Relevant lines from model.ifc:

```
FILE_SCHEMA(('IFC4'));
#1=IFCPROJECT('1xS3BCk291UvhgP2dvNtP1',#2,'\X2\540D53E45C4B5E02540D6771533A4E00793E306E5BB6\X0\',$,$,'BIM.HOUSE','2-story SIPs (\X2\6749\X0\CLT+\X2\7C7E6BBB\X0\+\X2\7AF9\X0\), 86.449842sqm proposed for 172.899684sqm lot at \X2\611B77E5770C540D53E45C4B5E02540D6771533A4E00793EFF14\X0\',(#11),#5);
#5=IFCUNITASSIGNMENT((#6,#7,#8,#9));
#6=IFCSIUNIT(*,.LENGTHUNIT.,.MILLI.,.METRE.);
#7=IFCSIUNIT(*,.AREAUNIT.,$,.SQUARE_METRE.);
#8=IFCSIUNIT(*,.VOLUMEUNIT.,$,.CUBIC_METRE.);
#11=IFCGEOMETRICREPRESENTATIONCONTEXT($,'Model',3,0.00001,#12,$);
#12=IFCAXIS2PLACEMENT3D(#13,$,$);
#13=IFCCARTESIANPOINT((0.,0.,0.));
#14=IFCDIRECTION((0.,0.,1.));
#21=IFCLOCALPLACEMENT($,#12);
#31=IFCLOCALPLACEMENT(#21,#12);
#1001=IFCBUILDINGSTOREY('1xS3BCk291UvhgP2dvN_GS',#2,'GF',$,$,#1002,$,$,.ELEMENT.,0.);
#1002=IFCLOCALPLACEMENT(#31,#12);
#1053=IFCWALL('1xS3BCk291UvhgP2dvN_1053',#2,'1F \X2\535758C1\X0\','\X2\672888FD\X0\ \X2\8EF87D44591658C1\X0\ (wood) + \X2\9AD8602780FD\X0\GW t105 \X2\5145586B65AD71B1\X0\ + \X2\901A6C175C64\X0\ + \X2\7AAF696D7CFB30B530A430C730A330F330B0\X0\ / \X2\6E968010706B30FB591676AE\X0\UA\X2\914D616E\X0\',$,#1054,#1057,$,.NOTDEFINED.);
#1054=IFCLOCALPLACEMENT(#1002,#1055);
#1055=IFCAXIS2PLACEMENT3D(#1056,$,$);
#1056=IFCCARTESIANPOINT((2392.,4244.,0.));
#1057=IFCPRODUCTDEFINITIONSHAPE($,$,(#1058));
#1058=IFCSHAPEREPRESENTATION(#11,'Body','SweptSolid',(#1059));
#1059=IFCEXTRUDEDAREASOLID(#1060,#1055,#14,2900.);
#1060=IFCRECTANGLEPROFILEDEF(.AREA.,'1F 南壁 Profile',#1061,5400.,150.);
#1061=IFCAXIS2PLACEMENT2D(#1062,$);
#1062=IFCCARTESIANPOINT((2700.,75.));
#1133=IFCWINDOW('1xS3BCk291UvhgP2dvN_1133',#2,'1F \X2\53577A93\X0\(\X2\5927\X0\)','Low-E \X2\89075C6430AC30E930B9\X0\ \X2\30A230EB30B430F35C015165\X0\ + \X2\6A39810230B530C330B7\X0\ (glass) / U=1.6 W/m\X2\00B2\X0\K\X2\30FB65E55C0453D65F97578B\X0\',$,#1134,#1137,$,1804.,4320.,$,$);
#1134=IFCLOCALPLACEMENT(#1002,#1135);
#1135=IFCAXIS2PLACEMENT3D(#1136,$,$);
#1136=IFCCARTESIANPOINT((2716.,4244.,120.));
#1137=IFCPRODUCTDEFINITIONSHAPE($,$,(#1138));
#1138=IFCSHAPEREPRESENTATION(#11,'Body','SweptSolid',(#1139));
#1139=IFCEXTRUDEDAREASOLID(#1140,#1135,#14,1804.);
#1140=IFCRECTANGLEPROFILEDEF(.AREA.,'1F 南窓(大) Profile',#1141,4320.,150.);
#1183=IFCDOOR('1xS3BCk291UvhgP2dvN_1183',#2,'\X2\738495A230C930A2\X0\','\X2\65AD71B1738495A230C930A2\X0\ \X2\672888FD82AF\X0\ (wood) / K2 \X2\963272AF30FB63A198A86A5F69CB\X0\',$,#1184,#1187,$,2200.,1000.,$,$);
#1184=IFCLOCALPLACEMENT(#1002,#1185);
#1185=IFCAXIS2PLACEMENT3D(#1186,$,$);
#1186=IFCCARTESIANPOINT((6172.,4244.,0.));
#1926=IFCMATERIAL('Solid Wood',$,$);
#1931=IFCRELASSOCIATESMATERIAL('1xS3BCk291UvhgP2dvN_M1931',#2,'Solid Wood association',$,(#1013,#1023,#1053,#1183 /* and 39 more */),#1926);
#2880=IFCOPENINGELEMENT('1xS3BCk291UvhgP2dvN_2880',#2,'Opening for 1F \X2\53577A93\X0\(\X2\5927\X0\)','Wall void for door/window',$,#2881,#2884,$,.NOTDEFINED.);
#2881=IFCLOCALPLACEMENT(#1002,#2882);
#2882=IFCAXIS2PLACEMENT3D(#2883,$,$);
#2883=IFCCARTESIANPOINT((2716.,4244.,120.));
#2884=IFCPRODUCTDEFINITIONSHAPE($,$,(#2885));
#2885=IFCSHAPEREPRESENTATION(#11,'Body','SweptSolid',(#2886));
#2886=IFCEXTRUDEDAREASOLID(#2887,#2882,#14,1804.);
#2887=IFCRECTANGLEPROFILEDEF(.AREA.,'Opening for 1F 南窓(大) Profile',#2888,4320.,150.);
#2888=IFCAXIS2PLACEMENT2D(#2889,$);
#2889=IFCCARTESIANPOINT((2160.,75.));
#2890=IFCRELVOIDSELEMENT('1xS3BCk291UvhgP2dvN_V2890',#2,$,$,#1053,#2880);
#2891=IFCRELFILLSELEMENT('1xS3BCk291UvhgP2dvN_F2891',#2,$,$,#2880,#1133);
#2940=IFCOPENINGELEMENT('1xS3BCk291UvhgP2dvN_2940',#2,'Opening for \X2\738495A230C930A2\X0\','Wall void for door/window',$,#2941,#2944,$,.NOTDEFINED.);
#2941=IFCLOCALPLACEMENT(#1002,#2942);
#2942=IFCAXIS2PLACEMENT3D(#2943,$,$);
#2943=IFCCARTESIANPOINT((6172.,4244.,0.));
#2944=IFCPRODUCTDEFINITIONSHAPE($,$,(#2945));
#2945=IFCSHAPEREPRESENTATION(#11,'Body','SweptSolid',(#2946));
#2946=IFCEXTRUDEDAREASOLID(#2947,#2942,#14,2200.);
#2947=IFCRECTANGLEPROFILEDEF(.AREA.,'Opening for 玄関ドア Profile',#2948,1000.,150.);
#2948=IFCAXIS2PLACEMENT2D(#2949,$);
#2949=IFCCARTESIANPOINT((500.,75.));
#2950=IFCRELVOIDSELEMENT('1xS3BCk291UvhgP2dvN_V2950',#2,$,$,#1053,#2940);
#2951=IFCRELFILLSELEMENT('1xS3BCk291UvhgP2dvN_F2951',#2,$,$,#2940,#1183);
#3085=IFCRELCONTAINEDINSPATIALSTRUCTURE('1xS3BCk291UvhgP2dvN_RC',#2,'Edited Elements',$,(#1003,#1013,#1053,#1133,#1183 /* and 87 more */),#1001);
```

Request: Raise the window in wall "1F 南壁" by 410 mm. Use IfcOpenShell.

```python
import numpy as np
import ifcopenshell
import ifcopenshell.api.geometry
import ifcopenshell.util.placement
import ifcopenshell.util.unit

model = ifcopenshell.open("model.ifc")
unit_scale = ifcopenshell.util.unit.calculate_unit_scale(model)

window = model.by_guid("1xS3BCk291UvhgP2dvN_1133")
opening = window.FillsVoids[0].RelatingOpeningElement
dz = 0.41 / unit_scale

shift = np.array([0.0, 0.0, dz])
# The window is not placed relative to its opening, so move both.
for product in (opening, window):
    matrix = ifcopenshell.util.placement.get_local_placement(product.ObjectPlacement)
    matrix[:3, 3] += shift
    ifcopenshell.api.geometry.edit_object_placement(model, product=product, matrix=matrix, is_si=False)

print(f"moved by {dz * unit_scale:+.3f} m")

model.write("model_edited.ifc")
```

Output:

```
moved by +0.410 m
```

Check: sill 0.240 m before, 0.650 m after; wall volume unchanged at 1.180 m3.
